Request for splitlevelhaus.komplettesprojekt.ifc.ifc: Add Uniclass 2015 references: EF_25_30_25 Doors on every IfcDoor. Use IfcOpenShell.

First a look at what the model holds.

```python
import ifcopenshell

model = ifcopenshell.open("splitlevelhaus.komplettesprojekt.ifc.ifc")
print(model.schema)
print("classifications:", [c.Name for c in model.by_type("IfcClassification")])
for ifc_class in ("IfcDoor", "IfcRoof", "IfcStair", "IfcWall", "IfcWindow"):
    print(ifc_class, len(model.by_type(ifc_class)))
```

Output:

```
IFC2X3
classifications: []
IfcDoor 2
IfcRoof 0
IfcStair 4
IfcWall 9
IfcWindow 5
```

```python
import ifcopenshell
import ifcopenshell.api.classification

model = ifcopenshell.open("splitlevelhaus.komplettesprojekt.ifc.ifc")

# IFC2X3 requires Source and Edition and has no link from the project to the system.
system = model.create_entity("IfcClassification", Source="NBS", Edition="2015", Name="Uniclass 2015")

codes = {
    "IfcDoor": ("EF_25_30_25", "Doors"),
}
for ifc_class, (code, name) in codes.items():
    products = model.by_type(ifc_class)
    ifcopenshell.api.classification.add_reference(
        model, products=products, classification=system, identification=code, name=name
    )
    print(code, len(products))

model.write("splitlevelhaus.komplettesprojekt.ifc_updated.ifc")
```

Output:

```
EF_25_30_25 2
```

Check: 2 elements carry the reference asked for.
